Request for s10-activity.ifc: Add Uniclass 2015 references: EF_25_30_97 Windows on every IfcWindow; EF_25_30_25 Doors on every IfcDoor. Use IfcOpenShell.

First a look at what the model holds.

```python
import ifcopenshell

model = ifcopenshell.open("s10-activity.ifc")
print(model.schema)
print("classifications:", [c.Name for c in model.by_type("IfcClassification")])
for ifc_class in ("IfcDoor", "IfcRoof", "IfcStair", "IfcWall", "IfcWindow"):
    print(ifc_class, len(model.by_type(ifc_class)))
```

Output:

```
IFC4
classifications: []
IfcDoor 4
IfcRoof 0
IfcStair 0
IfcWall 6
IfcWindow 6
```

```python
import ifcopenshell
import ifcopenshell.api.classification

model = ifcopenshell.open("s10-activity.ifc")

system = ifcopenshell.api.classification.add_classification(model, classification="Uniclass 2015")

codes = {
    "IfcWindow": ("EF_25_30_97", "Windows"),
    "IfcDoor": ("EF_25_30_25", "Doors"),
}
for ifc_class, (code, name) in codes.items():
    products = model.by_type(ifc_class)
    ifcopenshell.api.classification.add_reference(
        model, products=products, classification=system, identification=code, name=name
    )
    print(code, len(products))

model.write("s10-activity_edited.ifc")
```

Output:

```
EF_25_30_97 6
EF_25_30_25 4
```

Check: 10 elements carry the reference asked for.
